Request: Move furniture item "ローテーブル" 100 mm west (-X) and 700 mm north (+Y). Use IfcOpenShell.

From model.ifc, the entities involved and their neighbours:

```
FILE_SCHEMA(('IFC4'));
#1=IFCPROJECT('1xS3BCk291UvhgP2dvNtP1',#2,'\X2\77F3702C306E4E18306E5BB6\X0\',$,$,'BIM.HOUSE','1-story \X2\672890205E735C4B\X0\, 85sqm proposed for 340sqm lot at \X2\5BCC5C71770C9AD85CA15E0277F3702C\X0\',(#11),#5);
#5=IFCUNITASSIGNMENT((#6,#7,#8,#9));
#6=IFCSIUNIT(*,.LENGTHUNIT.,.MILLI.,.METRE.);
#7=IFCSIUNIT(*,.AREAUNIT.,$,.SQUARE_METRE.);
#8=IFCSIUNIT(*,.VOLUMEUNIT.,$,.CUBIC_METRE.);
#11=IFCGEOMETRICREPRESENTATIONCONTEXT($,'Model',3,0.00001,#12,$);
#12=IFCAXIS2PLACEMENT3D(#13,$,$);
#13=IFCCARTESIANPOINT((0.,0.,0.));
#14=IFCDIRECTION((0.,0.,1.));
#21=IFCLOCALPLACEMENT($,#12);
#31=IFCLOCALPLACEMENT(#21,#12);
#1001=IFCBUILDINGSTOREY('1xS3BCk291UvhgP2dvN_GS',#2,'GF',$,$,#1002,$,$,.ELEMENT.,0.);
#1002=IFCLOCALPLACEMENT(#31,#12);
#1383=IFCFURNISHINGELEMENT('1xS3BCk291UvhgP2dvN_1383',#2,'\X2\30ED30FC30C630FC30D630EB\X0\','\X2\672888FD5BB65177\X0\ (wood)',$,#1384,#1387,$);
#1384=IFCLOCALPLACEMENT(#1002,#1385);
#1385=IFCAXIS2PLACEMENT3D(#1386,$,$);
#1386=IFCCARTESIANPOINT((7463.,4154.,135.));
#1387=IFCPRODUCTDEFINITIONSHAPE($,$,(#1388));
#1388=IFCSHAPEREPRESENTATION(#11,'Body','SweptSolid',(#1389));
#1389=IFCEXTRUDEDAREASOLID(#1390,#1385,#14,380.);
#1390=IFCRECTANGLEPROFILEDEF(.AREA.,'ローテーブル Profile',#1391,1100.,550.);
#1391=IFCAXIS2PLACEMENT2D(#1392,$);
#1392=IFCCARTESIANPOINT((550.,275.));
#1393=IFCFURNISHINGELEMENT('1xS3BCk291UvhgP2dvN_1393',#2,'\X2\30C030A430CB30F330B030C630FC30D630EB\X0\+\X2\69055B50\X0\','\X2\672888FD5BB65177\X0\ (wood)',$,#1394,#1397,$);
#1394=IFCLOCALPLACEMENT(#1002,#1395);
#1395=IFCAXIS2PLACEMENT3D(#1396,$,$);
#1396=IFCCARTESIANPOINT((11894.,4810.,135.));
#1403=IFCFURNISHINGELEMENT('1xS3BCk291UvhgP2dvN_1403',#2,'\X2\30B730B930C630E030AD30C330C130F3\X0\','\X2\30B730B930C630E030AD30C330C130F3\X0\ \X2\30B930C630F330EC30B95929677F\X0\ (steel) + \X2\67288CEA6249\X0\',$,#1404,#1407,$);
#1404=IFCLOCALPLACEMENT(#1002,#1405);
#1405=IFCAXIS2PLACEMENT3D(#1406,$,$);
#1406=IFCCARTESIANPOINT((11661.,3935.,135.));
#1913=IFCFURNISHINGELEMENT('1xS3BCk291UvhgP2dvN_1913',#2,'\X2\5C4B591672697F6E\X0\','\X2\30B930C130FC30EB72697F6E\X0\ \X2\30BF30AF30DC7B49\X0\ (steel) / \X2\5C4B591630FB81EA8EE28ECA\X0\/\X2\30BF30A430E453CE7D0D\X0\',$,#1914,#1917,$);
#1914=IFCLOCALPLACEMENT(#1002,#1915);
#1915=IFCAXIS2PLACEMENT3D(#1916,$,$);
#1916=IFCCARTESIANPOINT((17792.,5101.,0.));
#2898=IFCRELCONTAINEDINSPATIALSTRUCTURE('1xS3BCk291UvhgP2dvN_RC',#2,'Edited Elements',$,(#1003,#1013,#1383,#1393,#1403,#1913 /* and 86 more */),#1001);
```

```python
import ifcopenshell
import ifcopenshell.api.geometry
import ifcopenshell.util.placement
import ifcopenshell.util.unit

model = ifcopenshell.open("model.ifc")
unit_scale = ifcopenshell.util.unit.calculate_unit_scale(model)

item = model.by_guid("1xS3BCk291UvhgP2dvN_1383")
matrix = ifcopenshell.util.placement.get_local_placement(item.ObjectPlacement)
matrix[0, 3] -= 0.1 / unit_scale
matrix[1, 3] += 0.7 / unit_scale
ifcopenshell.api.geometry.edit_object_placement(model, product=item, matrix=matrix, is_si=False)

print(ifcopenshell.util.placement.get_local_placement(item.ObjectPlacement).round(3) + 0.0)

model.write("model_rev.ifc")
```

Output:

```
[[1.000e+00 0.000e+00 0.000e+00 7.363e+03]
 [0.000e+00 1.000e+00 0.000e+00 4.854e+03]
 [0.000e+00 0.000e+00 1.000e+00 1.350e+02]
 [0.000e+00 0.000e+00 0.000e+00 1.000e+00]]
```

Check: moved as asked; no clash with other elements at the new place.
